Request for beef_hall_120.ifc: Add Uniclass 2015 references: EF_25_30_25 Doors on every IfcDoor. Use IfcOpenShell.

First a look at what the model holds.

```python
import ifcopenshell

model = ifcopenshell.open("beef_hall_120.ifc")
print(model.schema)
print("classifications:", [c.Name for c in model.by_type("IfcClassification")])
for ifc_class in ("IfcDoor", "IfcRoof", "IfcStair", "IfcWall", "IfcWindow"):
    print(ifc_class, len(model.by_type(ifc_class)))
```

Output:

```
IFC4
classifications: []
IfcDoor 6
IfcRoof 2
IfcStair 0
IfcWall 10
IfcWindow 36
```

```python
import ifcopenshell
import ifcopenshell.api.classification

model = ifcopenshell.open("beef_hall_120.ifc")

system = ifcopenshell.api.classification.add_classification(model, classification="Uniclass 2015")

codes = {
    "IfcDoor": ("EF_25_30_25", "Doors"),
}
for ifc_class, (code, name) in codes.items():
    products = model.by_type(ifc_class)
    ifcopenshell.api.classification.add_reference(
        model, products=products, classification=system, identification=code, name=name
    )
    print(code, len(products))

model.write("beef_hall_120_rev.ifc")
```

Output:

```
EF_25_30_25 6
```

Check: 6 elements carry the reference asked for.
